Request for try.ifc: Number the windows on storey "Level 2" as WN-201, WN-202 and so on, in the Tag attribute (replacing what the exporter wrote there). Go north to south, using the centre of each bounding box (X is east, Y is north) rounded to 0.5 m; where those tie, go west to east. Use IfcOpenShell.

First a look at what the model holds.

```python
import ifcopenshell
import ifcopenshell.util.element
import ifcopenshell.util.placement

model = ifcopenshell.open("try.ifc")
print(model.schema)
storey = next(s for s in model.by_type("IfcBuildingStorey") if s.Name == "Level 2")
windows = [e for e in ifcopenshell.util.element.get_decomposition(storey) if e.is_a("IfcWindow")]
for e in sorted(windows, key=lambda e: e.id()):
    origin = ifcopenshell.util.placement.get_local_placement(e.ObjectPlacement)[:3, 3]
    print(e.id(), e.Tag, e.Name, origin.round(2) + 0.0, sep=" | ")
```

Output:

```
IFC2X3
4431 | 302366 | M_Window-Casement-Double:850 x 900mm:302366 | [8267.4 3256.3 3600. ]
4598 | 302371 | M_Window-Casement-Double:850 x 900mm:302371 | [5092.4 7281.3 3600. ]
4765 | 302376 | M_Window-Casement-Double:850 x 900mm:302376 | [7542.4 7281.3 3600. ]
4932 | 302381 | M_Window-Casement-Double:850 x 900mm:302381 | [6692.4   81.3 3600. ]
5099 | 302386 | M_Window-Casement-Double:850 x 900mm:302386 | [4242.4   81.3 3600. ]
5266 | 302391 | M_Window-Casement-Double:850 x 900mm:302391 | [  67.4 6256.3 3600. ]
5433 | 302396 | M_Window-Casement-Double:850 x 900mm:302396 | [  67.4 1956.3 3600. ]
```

```python
import ifcopenshell
import ifcopenshell.geom
import ifcopenshell.util.element
import ifcopenshell.util.shape

model = ifcopenshell.open("try.ifc")
settings = ifcopenshell.geom.settings()
settings.set("use-world-coords", True)


def centre(element):
    shape = ifcopenshell.geom.create_shape(settings, element)
    return ifcopenshell.util.shape.get_bbox_centroid(shape.geometry)


storey = next(s for s in model.by_type("IfcBuildingStorey") if s.Name == "Level 2")
windows = [e for e in ifcopenshell.util.element.get_decomposition(storey) if e.is_a("IfcWindow")]

# Insertion points can sit at a corner or the storey origin, so sort by the geometry (in metres).
centres = {e: centre(e) for e in windows}
windows.sort(key=lambda e: (-round(centres[e][1] / 0.5), centres[e][0]))

for i, e in enumerate(windows, start=1):
    number = f"WN-2{i:02d}"
    e.Tag = number
    print(e.id(), number)

model.write("try_edited.ifc")
```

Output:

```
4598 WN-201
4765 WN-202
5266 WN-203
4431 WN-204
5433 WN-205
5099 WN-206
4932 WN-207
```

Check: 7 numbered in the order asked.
